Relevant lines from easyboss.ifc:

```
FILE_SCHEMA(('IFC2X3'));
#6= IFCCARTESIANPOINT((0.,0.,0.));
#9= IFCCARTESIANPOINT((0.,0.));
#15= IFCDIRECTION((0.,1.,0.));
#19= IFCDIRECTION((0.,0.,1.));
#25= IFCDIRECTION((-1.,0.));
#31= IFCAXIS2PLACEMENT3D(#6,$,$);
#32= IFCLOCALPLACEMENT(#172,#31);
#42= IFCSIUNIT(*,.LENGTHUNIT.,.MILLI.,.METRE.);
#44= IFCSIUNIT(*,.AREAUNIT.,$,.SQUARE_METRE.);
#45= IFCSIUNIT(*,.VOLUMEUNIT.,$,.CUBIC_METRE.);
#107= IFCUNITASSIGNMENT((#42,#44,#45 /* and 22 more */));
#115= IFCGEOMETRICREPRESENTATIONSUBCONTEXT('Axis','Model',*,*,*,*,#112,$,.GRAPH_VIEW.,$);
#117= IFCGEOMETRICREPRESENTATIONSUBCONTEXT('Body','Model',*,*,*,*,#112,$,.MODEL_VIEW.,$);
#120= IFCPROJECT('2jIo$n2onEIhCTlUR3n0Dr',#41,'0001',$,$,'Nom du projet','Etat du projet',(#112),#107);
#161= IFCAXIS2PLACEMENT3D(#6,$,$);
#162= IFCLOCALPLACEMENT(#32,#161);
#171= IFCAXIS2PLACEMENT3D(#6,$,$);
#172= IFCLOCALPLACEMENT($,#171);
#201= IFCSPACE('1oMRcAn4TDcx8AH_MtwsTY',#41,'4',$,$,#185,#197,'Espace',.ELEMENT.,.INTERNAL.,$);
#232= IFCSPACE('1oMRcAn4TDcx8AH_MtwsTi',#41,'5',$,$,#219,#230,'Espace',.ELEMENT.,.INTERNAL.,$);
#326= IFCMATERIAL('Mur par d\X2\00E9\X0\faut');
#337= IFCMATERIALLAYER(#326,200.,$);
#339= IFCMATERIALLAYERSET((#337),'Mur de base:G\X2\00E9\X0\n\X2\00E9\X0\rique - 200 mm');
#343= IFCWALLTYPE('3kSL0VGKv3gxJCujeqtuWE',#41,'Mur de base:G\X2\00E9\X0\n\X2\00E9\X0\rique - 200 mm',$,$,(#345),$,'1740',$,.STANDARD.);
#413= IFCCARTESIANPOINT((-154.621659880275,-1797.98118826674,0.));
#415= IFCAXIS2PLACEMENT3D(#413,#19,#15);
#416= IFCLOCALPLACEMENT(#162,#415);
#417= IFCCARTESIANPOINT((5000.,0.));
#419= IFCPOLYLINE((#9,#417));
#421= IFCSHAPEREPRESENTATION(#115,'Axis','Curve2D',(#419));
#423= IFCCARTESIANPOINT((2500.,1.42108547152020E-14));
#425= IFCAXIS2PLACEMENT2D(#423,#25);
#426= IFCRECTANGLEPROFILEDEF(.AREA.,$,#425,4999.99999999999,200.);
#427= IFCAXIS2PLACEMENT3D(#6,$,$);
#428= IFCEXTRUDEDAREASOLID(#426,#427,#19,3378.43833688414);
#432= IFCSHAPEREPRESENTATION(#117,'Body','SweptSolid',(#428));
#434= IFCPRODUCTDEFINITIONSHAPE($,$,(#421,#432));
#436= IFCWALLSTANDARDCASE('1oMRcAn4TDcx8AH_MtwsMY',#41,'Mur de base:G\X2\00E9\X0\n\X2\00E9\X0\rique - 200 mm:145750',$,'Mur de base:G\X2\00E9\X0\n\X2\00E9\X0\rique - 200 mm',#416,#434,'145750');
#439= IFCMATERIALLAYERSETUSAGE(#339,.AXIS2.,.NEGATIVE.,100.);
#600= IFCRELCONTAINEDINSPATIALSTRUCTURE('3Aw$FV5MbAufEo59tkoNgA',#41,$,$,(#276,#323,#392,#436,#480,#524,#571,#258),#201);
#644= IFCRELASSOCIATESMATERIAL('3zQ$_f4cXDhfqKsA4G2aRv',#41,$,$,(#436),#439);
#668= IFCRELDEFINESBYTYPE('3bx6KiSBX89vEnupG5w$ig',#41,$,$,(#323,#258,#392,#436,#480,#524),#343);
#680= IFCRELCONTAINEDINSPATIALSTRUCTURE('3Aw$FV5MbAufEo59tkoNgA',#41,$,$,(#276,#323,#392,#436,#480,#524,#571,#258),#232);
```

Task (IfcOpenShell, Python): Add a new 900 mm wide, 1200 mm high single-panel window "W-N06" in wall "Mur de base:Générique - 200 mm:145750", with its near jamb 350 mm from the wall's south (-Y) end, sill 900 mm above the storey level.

```python
import numpy as np
import ifcopenshell
import ifcopenshell.api.feature
import ifcopenshell.api.geometry
import ifcopenshell.api.root
import ifcopenshell.api.spatial
import ifcopenshell.api.type
import ifcopenshell.geom
import ifcopenshell.util.element
import ifcopenshell.util.placement
import ifcopenshell.util.representation
import ifcopenshell.util.shape
import ifcopenshell.util.unit

model = ifcopenshell.open("easyboss.ifc")
unit_scale = ifcopenshell.util.unit.calculate_unit_scale(model)
settings = ifcopenshell.geom.settings()


def volume(element):
    """Net volume in cubic metres, openings subtracted."""
    shape = ifcopenshell.geom.create_shape(settings, element)
    return ifcopenshell.util.shape.get_volume(shape.geometry)


wall = model.by_id(436)
storey = ifcopenshell.util.element.get_container(wall, ifc_class="IfcBuildingStorey")
context = ifcopenshell.util.representation.get_context(model, "Model", "Body", "MODEL_VIEW")
before = volume(wall)

width, height, from_end, sill = 0.9, 1.2, 0.35, 0.9  # metres

# The wall runs along its own X axis, and the end named is its -X end.
wall_shape = ifcopenshell.geom.create_shape(settings, wall)
x, y, z = ifcopenshell.util.shape.get_vertices(wall_shape.geometry).T
start = x.min() + from_end
face, thickness = float(y.min()), float(y.max() - y.min())
wall_matrix = ifcopenshell.util.placement.get_local_placement(wall.ObjectPlacement)
level = ifcopenshell.util.placement.get_local_placement(storey.ObjectPlacement)[2, 3]


def in_wall(x, y):
    """Placement at x, y metres in the wall's axes, at sill height."""
    matrix = wall_matrix.copy()
    matrix[:, 3] = wall_matrix @ np.array([x / unit_scale, y / unit_scale, 0.0, 1.0])
    matrix[2, 3] = level + sill / unit_scale
    return matrix


# Opening: a box that overshoots both wall faces by 50 mm.
opening = ifcopenshell.api.root.create_entity(model, ifc_class="IfcOpeningElement")
box = ifcopenshell.api.geometry.add_wall_representation(
    model, context=context, length=width, height=height, thickness=thickness + 0.1
)
ifcopenshell.api.geometry.assign_representation(model, product=opening, representation=box)
ifcopenshell.api.geometry.edit_object_placement(model, product=opening, matrix=in_wall(start, face - 0.05), is_si=False)
ifcopenshell.api.feature.add_feature(model, feature=opening, element=wall)

window = ifcopenshell.api.root.create_entity(model, ifc_class="IfcWindow", name="W-N06")
window.OverallWidth, window.OverallHeight = width / unit_scale, height / unit_scale
body = ifcopenshell.api.geometry.add_window_representation(
    model,
    context=context,
    overall_width=window.OverallWidth,
    overall_height=window.OverallHeight,
    partition_type="SINGLE_PANEL",
)
ifcopenshell.api.geometry.assign_representation(model, product=window, representation=body)
ifcopenshell.api.spatial.assign_container(model, products=[window], relating_structure=storey)
fills = ifcopenshell.api.feature.add_filling(model, opening=opening, element=window)
fills.OwnerHistory = window.OwnerHistory  # required in IFC2X3

# IFC2X3 keeps the operation on the window style.
style = ifcopenshell.api.root.create_entity(model, ifc_class="IfcWindowStyle", name="W-N06")
style.OperationType, style.ConstructionType = "SINGLE_PANEL", "NOTDEFINED"
style.ParameterTakesPrecedence = style.Sizeable = False
ifcopenshell.api.type.assign_type(model, related_objects=[window], relating_type=style)

# Centre the window in the wall's thickness.
ifcopenshell.api.geometry.edit_object_placement(model, product=window, matrix=in_wall(start, face), is_si=False)
window_shape = ifcopenshell.geom.create_shape(settings, window)
depth = ifcopenshell.util.shape.get_vertices(window_shape.geometry)[:, 1]
offset = face + thickness / 2 - (depth.min() + depth.max()) / 2
ifcopenshell.api.geometry.edit_object_placement(model, product=window, matrix=in_wall(start, offset), is_si=False)

after = volume(wall)

print(f"wall volume {before:.3f} -> {after:.3f} m3")

model.write("easyboss-out.ifc")
```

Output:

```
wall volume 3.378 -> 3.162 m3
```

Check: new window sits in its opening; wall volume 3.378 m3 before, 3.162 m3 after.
